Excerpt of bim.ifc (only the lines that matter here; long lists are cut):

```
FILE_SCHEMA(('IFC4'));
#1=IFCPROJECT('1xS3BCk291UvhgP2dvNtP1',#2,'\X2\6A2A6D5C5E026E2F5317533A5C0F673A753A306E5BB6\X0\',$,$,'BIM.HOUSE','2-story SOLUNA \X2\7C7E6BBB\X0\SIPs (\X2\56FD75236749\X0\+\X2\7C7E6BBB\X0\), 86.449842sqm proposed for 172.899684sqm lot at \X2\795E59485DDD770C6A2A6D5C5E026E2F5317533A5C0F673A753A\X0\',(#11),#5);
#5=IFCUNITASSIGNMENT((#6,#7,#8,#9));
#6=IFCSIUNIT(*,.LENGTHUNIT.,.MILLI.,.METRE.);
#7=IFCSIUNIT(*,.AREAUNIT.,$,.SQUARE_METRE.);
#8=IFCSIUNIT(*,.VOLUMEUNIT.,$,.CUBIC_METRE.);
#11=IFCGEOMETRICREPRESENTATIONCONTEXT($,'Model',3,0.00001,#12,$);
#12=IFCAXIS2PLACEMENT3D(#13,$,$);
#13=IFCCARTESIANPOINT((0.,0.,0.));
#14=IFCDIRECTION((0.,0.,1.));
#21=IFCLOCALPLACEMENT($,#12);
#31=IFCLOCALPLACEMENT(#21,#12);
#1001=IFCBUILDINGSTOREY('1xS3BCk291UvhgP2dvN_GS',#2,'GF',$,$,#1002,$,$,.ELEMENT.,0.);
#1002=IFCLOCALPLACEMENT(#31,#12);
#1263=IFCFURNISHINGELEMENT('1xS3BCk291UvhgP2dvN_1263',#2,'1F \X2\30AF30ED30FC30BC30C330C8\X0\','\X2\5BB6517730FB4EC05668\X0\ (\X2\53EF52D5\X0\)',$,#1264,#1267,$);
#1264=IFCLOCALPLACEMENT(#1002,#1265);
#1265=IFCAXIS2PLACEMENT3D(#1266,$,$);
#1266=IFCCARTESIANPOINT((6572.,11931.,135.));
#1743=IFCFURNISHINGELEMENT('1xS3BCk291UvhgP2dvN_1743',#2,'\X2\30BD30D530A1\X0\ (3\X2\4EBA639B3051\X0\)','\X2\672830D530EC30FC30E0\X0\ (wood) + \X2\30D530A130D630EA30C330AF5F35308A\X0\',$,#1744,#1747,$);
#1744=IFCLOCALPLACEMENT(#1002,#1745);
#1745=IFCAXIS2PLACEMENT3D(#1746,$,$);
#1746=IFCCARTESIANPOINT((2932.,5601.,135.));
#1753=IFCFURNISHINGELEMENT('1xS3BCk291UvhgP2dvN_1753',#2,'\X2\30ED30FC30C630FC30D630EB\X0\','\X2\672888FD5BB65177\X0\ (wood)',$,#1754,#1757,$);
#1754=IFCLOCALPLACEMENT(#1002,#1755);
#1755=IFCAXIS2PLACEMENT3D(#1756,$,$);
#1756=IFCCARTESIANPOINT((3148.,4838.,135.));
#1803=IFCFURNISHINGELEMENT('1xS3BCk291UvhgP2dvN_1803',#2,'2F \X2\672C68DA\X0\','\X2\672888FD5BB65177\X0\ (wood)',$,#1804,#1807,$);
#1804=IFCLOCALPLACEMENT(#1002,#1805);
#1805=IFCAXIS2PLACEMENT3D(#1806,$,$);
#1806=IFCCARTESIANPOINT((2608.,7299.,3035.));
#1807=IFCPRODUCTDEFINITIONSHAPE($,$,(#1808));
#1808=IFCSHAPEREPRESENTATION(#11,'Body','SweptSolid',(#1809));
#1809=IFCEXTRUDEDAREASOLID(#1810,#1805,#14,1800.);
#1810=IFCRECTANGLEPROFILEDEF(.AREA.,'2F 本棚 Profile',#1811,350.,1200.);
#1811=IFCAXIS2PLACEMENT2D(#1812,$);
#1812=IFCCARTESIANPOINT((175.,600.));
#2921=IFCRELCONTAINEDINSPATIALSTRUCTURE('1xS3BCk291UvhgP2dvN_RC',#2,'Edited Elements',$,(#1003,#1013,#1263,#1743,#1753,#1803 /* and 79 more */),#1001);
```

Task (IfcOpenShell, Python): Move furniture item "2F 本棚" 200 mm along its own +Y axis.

```python
import ifcopenshell
import ifcopenshell.api.geometry
import ifcopenshell.util.placement
import ifcopenshell.util.unit

model = ifcopenshell.open("bim.ifc")
unit_scale = ifcopenshell.util.unit.calculate_unit_scale(model)

item = model.by_guid("1xS3BCk291UvhgP2dvN_1803")
matrix = ifcopenshell.util.placement.get_local_placement(item.ObjectPlacement)
matrix[:3, 3] += matrix[:3, 1] * 0.2 / unit_scale
ifcopenshell.api.geometry.edit_object_placement(model, product=item, matrix=matrix, is_si=False)

print(ifcopenshell.util.placement.get_local_placement(item.ObjectPlacement).round(3) + 0.0)

model.write("bim_updated.ifc")
```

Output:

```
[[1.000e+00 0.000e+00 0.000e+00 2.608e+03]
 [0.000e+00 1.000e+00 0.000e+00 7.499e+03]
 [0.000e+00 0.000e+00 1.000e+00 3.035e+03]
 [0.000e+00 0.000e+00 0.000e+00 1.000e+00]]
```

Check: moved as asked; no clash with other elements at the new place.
